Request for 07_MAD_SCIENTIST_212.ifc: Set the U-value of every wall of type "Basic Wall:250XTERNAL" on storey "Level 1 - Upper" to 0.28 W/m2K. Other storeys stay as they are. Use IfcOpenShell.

First a look at what the model holds.

```python
import ifcopenshell
import ifcopenshell.util.element

model = ifcopenshell.open("07_MAD_SCIENTIST_212.ifc")
print(model.schema)
storey = next(s for s in model.by_type("IfcBuildingStorey") if s.Name == "Level 1 - Upper")
walls = [e for e in ifcopenshell.util.element.get_decomposition(storey) if e.is_a("IfcWall")]
seen = {}
for e in walls:
    element_type = ifcopenshell.util.element.get_type(e)
    key = (element_type.Name if element_type != e and element_type else None, ifcopenshell.util.element.get_pset(e, "Pset_WallCommon", "ThermalTransmittance"))
    seen[key] = seen.get(key, 0) + 1
for (name, value), count in sorted(seen.items(), key=str):
    print(count, "x", name, "|", value)
```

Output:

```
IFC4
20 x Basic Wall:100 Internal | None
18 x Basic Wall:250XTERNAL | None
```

```python
import ifcopenshell
import ifcopenshell.api.pset
import ifcopenshell.util.element

model = ifcopenshell.open("07_MAD_SCIENTIST_212.ifc")

storey = next(s for s in model.by_type("IfcBuildingStorey") if s.Name == "Level 1 - Upper")
walls = [e for e in ifcopenshell.util.element.get_decomposition(storey) if e.is_a("IfcWall")]

count = 0
for e in walls:
    element_type = ifcopenshell.util.element.get_type(e)
    if element_type in (None, e) or element_type.Name != "Basic Wall:250XTERNAL":
        continue
    # add_pset returns the element's existing set when there is one.
    pset = ifcopenshell.api.pset.add_pset(model, product=e, name="Pset_WallCommon")
    ifcopenshell.api.pset.edit_pset(model, pset=pset, properties={"ThermalTransmittance": 0.28})
    count += 1

print(count, "walls updated")

model.write("07_MAD_SCIENTIST_212_edited.ifc")
```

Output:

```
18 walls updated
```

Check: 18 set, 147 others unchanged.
